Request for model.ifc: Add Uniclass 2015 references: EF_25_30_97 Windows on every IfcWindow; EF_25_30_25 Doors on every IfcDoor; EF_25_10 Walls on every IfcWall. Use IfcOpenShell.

First a look at what the model holds.

```python
import ifcopenshell

model = ifcopenshell.open("model.ifc")
print(model.schema)
print("classifications:", [c.Name for c in model.by_type("IfcClassification")])
for ifc_class in ("IfcDoor", "IfcRoof", "IfcStair", "IfcWall", "IfcWindow"):
    print(ifc_class, len(model.by_type(ifc_class)))
```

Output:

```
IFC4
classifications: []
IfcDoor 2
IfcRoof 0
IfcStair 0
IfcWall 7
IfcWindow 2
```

```python
import ifcopenshell
import ifcopenshell.api.classification

model = ifcopenshell.open("model.ifc")

system = ifcopenshell.api.classification.add_classification(model, classification="Uniclass 2015")

codes = {
    "IfcWindow": ("EF_25_30_97", "Windows"),
    "IfcDoor": ("EF_25_30_25", "Doors"),
    "IfcWall": ("EF_25_10", "Walls"),
}
for ifc_class, (code, name) in codes.items():
    products = model.by_type(ifc_class)
    ifcopenshell.api.classification.add_reference(
        model, products=products, classification=system, identification=code, name=name
    )
    print(code, len(products))

model.write("model_v2.ifc")
```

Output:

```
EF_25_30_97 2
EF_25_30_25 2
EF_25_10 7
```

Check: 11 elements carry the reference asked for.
